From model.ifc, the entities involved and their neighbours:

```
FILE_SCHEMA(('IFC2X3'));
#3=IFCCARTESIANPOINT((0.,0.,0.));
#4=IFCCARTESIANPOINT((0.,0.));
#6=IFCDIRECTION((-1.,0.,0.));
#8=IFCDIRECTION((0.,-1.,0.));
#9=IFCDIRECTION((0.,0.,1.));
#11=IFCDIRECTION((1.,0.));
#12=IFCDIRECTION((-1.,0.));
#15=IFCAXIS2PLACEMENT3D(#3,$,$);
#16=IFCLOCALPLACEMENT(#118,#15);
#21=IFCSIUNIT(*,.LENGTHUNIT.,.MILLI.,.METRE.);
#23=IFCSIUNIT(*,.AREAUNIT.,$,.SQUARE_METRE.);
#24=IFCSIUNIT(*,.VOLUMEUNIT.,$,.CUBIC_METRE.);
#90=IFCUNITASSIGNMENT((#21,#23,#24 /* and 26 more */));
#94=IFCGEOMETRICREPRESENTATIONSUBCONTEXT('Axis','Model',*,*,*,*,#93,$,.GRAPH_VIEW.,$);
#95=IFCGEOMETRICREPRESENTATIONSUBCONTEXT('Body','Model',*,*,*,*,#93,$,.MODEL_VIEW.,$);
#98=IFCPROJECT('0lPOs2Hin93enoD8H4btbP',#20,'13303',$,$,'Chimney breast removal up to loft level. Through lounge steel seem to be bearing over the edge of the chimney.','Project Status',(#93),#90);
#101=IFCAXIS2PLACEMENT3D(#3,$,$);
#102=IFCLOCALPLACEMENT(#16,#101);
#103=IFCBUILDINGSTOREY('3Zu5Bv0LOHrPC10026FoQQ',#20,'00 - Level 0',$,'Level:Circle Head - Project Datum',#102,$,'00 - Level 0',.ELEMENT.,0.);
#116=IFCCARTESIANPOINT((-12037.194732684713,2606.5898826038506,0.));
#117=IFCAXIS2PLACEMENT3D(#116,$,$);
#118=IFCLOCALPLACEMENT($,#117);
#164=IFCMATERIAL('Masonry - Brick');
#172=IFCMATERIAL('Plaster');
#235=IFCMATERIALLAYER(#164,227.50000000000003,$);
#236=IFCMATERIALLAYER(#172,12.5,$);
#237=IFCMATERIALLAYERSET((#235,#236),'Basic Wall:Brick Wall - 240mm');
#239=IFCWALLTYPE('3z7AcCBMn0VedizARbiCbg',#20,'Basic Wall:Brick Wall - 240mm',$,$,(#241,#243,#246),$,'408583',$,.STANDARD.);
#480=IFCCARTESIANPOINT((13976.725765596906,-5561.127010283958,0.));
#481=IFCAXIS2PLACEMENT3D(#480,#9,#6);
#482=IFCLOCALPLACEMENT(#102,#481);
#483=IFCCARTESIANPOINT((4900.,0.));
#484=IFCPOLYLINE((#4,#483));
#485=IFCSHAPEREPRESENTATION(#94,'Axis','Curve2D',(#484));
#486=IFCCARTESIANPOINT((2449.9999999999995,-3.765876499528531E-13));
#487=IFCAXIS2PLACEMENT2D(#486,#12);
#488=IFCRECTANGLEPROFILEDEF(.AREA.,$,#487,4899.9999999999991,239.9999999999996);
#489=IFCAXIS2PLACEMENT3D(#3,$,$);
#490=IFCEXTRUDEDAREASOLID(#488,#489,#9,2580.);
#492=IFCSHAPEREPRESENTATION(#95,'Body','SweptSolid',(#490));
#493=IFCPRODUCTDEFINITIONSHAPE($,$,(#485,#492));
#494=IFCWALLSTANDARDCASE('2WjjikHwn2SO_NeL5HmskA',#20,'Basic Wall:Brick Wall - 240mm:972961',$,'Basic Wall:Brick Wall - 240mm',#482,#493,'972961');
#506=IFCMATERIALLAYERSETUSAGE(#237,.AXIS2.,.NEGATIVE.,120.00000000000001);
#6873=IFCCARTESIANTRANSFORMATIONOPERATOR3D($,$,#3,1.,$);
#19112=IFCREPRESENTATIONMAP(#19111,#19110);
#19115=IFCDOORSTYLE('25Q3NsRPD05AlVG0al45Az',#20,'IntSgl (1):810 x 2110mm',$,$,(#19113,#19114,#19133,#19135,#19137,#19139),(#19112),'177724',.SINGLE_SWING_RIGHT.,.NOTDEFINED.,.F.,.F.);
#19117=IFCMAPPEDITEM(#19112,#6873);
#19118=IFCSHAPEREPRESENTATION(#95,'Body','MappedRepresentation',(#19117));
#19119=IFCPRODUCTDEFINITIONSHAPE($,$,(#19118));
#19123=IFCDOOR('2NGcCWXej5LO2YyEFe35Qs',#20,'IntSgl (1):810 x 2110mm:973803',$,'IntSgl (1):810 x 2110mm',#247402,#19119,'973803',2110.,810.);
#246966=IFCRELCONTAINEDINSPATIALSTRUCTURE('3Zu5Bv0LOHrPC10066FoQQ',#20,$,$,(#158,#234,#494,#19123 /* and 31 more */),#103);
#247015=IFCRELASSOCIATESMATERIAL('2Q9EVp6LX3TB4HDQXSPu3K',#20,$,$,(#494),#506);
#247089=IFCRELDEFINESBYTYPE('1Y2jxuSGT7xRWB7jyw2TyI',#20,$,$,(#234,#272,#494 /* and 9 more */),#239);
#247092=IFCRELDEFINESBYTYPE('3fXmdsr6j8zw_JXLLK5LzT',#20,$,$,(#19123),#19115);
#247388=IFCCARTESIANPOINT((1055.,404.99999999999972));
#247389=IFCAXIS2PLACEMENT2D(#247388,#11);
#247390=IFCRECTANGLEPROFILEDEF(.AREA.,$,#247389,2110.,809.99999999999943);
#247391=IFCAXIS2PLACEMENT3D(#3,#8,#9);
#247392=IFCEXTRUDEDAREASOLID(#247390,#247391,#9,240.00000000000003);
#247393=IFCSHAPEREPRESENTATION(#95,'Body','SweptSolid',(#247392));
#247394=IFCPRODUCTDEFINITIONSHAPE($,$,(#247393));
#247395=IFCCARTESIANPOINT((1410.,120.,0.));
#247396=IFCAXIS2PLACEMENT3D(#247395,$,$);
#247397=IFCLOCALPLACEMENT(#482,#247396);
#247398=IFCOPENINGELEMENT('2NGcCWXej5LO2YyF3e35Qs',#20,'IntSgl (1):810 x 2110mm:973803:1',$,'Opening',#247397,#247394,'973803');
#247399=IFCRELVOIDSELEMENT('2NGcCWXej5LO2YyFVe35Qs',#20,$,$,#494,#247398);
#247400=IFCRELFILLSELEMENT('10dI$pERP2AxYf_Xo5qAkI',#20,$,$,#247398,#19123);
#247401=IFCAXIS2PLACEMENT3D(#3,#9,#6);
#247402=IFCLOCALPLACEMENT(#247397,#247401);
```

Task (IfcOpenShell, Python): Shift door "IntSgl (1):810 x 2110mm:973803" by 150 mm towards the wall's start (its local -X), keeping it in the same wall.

```python
import ifcopenshell
import ifcopenshell.api.geometry
import ifcopenshell.util.placement
import ifcopenshell.util.unit

model = ifcopenshell.open("model.ifc")
unit_scale = ifcopenshell.util.unit.calculate_unit_scale(model)

door = model.by_guid("2NGcCWXej5LO2YyEFe35Qs")
opening = door.FillsVoids[0].RelatingOpeningElement
wall = opening.VoidsElements[0].RelatingBuildingElement

wall_matrix = ifcopenshell.util.placement.get_local_placement(wall.ObjectPlacement)
shift = wall_matrix[:3, 0] * -0.15 / unit_scale
before = ifcopenshell.util.placement.get_local_placement(door.ObjectPlacement)[:3, 3].copy()

# The door is placed relative to its opening, so it follows when the opening moves.
matrix = ifcopenshell.util.placement.get_local_placement(opening.ObjectPlacement)
matrix[:3, 3] += shift
ifcopenshell.api.geometry.edit_object_placement(
    model, product=opening, matrix=matrix, is_si=False, should_transform_children=True
)

after = ifcopenshell.util.placement.get_local_placement(door.ObjectPlacement)[:3, 3]
print("door moved by", (after - before).round(3) + 0.0)

model.write("model-out.ifc")
```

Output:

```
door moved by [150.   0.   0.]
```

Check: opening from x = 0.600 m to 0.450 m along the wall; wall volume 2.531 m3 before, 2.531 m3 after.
